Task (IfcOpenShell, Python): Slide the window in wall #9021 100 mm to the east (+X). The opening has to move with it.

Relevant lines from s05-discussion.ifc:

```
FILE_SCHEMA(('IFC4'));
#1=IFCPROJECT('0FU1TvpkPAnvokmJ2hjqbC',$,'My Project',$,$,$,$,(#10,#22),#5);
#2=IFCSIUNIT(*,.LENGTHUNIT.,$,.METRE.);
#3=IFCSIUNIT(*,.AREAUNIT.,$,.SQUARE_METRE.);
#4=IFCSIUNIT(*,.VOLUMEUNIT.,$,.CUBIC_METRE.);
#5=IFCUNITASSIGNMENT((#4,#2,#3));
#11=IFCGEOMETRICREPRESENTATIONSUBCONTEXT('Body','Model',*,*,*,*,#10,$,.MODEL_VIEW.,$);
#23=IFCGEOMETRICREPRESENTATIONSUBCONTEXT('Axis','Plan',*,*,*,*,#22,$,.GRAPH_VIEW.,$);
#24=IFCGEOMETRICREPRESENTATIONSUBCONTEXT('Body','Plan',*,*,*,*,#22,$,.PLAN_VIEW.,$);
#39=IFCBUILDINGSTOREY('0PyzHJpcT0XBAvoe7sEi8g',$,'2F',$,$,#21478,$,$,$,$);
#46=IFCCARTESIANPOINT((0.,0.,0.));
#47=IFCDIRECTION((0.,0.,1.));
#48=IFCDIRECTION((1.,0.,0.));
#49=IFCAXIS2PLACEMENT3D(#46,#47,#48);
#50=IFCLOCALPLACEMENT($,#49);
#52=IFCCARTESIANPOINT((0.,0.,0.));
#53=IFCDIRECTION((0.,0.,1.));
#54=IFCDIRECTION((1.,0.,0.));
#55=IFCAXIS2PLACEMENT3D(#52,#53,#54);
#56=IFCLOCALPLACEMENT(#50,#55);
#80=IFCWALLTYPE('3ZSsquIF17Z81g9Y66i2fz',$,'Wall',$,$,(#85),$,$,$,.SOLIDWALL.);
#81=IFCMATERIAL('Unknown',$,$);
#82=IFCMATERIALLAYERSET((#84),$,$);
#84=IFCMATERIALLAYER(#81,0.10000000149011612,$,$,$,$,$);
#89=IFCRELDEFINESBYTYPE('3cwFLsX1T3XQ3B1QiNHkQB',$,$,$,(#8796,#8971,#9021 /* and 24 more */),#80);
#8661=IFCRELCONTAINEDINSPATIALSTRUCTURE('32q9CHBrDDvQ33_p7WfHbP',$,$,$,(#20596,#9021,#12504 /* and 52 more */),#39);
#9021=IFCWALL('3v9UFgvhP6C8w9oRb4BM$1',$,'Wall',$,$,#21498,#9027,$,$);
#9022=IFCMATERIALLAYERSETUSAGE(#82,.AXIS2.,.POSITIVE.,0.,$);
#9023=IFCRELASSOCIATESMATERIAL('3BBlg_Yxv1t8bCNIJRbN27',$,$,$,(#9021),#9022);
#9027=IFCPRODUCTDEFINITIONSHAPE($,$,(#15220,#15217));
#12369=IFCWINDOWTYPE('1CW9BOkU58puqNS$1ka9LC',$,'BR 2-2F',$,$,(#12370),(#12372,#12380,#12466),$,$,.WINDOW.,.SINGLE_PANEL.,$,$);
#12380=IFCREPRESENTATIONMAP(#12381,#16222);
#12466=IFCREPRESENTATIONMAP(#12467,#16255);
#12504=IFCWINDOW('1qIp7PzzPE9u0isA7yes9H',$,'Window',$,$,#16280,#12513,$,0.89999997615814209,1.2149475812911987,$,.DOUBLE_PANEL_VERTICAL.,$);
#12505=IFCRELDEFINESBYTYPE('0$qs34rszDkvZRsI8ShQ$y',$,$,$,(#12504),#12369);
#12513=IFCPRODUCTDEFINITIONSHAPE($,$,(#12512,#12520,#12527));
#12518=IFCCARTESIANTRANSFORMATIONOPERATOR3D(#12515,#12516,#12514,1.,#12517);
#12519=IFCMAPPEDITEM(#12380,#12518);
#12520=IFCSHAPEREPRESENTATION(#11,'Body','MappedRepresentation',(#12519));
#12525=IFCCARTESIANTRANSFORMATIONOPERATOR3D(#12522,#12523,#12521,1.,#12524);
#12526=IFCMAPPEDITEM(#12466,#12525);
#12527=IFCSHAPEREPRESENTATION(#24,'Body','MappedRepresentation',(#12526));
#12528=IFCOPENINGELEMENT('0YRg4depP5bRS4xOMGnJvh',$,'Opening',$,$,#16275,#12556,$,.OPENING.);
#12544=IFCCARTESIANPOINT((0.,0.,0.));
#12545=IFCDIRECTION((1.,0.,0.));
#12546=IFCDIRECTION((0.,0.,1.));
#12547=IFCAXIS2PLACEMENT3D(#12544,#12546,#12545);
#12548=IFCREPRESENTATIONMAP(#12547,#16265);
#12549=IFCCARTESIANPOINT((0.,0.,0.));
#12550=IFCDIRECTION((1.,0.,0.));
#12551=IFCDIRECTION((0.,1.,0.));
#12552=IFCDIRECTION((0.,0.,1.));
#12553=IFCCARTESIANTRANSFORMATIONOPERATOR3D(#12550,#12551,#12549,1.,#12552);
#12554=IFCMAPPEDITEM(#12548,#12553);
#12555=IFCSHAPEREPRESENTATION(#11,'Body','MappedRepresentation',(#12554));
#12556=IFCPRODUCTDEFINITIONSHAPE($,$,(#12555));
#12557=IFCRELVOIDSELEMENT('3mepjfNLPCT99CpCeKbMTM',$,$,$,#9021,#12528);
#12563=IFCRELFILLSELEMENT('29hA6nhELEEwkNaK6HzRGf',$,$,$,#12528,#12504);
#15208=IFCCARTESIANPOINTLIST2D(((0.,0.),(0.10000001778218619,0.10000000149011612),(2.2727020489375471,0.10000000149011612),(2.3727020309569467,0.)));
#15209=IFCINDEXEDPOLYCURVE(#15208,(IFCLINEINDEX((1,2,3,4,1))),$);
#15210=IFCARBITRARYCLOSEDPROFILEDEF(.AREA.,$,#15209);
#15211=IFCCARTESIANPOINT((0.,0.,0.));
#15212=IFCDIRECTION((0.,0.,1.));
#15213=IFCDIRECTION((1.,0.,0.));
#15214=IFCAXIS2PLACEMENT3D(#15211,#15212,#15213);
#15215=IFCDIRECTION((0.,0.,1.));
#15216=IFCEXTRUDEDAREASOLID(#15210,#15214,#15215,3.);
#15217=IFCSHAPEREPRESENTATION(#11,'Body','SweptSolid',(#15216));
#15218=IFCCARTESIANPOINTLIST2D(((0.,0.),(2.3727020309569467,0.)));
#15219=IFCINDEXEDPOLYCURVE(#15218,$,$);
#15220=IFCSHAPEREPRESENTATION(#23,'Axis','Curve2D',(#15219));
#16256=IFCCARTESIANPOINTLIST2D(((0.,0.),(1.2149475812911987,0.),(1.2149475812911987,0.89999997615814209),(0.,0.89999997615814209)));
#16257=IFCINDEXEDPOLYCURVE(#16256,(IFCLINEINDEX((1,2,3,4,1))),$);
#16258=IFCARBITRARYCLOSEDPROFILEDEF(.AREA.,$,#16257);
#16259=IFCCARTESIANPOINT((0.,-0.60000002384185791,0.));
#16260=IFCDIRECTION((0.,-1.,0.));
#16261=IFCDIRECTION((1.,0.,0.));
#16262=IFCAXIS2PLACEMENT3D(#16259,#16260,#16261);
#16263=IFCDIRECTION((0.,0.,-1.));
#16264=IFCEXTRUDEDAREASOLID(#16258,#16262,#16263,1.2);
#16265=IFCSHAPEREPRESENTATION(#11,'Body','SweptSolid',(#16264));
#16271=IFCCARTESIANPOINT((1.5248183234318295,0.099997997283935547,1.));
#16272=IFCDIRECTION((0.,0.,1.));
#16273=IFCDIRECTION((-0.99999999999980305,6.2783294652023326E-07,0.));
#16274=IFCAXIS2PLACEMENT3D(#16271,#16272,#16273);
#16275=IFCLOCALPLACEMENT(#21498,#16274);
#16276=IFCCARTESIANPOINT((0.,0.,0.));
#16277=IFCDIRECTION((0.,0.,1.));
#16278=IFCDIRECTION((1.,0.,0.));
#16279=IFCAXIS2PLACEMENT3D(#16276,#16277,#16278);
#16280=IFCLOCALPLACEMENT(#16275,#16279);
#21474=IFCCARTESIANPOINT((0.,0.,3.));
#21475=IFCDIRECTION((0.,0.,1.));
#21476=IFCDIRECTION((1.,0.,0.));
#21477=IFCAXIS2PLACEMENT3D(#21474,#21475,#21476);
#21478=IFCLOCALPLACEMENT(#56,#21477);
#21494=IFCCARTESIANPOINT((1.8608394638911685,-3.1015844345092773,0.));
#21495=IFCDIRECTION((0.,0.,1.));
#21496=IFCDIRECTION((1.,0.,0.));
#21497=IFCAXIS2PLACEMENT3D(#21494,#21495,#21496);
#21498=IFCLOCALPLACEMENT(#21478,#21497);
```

```python
import ifcopenshell
import ifcopenshell.api.geometry
import ifcopenshell.util.placement
import ifcopenshell.util.unit

model = ifcopenshell.open("s05-discussion.ifc")
unit_scale = ifcopenshell.util.unit.calculate_unit_scale(model)

window = model.by_id(12504)
opening = window.FillsVoids[0].RelatingOpeningElement
wall = opening.VoidsElements[0].RelatingBuildingElement

wall_matrix = ifcopenshell.util.placement.get_local_placement(wall.ObjectPlacement)
shift = wall_matrix[:3, 0] * 0.1 / unit_scale
before = ifcopenshell.util.placement.get_local_placement(window.ObjectPlacement)[:3, 3].copy()

# The window is placed relative to its opening, so it follows when the opening moves.
matrix = ifcopenshell.util.placement.get_local_placement(opening.ObjectPlacement)
matrix[:3, 3] += shift
ifcopenshell.api.geometry.edit_object_placement(
    model, product=opening, matrix=matrix, is_si=False, should_transform_children=True
)

after = ifcopenshell.util.placement.get_local_placement(window.ObjectPlacement)[:3, 3]
print("window moved by", (after - before).round(3) + 0.0)

model.write("s05-discussion_updated.ifc")
```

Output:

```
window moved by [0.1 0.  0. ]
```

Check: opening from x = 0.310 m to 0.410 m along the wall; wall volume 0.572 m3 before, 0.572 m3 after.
